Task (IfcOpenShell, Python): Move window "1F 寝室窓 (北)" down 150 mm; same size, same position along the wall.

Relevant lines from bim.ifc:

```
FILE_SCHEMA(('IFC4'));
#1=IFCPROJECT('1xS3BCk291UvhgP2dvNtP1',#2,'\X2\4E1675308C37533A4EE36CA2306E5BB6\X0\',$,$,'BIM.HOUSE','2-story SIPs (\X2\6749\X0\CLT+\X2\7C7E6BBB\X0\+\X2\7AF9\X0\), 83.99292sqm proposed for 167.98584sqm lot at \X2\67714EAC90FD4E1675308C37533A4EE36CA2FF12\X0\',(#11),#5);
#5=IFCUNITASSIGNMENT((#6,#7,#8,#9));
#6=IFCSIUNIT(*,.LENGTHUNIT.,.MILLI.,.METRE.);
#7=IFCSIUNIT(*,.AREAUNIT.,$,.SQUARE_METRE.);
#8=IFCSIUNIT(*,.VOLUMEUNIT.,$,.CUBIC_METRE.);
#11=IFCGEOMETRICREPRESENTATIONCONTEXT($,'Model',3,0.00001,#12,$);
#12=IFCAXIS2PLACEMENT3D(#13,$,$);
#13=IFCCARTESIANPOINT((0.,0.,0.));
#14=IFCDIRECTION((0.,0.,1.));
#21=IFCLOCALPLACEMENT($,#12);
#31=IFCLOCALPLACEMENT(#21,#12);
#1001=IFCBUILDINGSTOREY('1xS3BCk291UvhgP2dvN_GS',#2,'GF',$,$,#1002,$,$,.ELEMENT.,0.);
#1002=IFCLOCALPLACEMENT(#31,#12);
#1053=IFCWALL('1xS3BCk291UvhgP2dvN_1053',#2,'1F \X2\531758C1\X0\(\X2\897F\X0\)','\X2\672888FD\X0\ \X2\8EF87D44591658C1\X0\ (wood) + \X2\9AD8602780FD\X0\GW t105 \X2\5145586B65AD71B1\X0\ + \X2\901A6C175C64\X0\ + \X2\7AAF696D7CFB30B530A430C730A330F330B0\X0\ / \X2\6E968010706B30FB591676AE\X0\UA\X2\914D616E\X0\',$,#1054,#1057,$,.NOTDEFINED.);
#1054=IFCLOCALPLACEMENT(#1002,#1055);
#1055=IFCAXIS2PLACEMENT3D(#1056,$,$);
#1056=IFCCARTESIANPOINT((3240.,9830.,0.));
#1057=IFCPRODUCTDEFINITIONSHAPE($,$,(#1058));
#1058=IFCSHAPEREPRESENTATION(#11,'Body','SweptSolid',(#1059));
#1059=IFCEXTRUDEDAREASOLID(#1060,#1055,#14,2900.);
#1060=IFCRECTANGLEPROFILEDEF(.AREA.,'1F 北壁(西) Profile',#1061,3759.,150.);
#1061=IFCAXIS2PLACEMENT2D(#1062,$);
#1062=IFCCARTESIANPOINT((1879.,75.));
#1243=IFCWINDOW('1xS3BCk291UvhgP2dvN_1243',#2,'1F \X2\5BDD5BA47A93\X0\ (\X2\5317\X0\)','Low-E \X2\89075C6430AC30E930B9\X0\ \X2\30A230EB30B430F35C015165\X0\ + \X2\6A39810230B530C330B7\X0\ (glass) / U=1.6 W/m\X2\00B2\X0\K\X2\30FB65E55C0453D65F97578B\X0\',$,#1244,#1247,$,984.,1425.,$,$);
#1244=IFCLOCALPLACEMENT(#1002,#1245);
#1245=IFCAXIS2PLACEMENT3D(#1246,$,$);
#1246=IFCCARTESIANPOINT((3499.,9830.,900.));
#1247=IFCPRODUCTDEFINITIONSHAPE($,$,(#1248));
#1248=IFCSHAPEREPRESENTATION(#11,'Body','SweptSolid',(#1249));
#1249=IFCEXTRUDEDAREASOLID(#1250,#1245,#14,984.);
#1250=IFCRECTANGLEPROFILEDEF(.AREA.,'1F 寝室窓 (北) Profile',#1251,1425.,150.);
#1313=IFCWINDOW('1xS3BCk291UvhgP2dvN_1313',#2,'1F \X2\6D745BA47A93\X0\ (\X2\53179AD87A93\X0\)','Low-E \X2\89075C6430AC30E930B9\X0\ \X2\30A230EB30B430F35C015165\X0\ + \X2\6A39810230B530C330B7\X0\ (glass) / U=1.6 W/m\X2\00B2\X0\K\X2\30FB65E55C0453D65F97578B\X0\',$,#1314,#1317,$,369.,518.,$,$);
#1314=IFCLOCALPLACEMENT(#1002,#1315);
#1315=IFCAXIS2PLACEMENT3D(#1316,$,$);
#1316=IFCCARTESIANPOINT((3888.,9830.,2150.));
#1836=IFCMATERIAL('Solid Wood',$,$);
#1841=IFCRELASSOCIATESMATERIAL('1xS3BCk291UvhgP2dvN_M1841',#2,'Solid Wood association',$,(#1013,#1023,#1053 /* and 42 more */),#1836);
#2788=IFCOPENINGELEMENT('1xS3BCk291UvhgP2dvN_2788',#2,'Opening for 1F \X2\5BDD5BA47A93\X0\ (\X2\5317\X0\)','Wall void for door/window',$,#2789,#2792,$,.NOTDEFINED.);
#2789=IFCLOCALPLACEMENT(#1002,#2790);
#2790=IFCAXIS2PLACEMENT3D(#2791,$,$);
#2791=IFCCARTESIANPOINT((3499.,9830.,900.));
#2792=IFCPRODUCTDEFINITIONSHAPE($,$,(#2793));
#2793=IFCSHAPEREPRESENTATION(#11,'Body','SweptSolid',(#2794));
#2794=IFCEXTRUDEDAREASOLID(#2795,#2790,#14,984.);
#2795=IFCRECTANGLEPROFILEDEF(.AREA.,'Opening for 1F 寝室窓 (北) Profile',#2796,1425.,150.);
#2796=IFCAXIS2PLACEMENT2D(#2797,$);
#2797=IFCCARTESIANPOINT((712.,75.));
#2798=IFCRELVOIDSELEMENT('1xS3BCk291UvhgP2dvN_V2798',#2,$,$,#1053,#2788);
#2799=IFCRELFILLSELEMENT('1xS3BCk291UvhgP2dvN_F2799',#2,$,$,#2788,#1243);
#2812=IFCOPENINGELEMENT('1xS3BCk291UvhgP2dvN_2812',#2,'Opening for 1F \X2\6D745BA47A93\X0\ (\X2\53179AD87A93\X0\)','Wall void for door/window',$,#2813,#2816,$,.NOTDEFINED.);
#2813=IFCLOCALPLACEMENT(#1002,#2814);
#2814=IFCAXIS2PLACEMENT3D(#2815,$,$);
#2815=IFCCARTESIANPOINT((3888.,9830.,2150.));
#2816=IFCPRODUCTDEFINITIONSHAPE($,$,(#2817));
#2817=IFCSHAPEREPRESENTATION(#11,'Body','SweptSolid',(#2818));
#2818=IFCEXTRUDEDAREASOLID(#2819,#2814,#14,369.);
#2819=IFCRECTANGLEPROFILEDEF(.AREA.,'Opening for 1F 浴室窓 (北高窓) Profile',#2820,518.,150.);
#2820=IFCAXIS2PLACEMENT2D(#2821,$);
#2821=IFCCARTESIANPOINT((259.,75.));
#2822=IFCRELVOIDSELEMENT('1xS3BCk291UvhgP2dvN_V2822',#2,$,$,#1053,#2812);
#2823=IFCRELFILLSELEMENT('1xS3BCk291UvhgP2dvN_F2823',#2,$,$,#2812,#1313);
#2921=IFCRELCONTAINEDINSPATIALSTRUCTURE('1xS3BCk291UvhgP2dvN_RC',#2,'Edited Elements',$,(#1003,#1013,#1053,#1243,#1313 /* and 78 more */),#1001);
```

```python
import numpy as np
import ifcopenshell
import ifcopenshell.api.geometry
import ifcopenshell.util.placement
import ifcopenshell.util.unit

model = ifcopenshell.open("bim.ifc")
unit_scale = ifcopenshell.util.unit.calculate_unit_scale(model)

window = model.by_guid("1xS3BCk291UvhgP2dvN_1243")
opening = window.FillsVoids[0].RelatingOpeningElement
dz = -0.15 / unit_scale

shift = np.array([0.0, 0.0, dz])
# The window is not placed relative to its opening, so move both.
for product in (opening, window):
    matrix = ifcopenshell.util.placement.get_local_placement(product.ObjectPlacement)
    matrix[:3, 3] += shift
    ifcopenshell.api.geometry.edit_object_placement(model, product=product, matrix=matrix, is_si=False)

print(f"moved by {dz * unit_scale:+.3f} m")

model.write("bim_updated.ifc")
```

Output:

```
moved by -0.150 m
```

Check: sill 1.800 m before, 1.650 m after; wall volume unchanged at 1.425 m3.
